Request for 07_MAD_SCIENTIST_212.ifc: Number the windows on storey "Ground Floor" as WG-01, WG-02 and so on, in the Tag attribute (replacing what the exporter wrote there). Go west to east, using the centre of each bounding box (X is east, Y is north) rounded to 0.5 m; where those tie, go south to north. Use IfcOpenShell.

First a look at what the model holds.

```python
import ifcopenshell
import ifcopenshell.util.element
import ifcopenshell.util.placement

model = ifcopenshell.open("07_MAD_SCIENTIST_212.ifc")
print(model.schema)
storey = next(s for s in model.by_type("IfcBuildingStorey") if s.Name == "Ground Floor")
windows = [e for e in ifcopenshell.util.element.get_decomposition(storey) if e.is_a("IfcWindow")]
for e in sorted(windows, key=lambda e: e.id()):
    origin = ifcopenshell.util.placement.get_local_placement(e.ObjectPlacement)[:3, 3]
    print(e.id(), e.Tag, e.Name, origin.round(2) + 0.0, sep=" | ")
```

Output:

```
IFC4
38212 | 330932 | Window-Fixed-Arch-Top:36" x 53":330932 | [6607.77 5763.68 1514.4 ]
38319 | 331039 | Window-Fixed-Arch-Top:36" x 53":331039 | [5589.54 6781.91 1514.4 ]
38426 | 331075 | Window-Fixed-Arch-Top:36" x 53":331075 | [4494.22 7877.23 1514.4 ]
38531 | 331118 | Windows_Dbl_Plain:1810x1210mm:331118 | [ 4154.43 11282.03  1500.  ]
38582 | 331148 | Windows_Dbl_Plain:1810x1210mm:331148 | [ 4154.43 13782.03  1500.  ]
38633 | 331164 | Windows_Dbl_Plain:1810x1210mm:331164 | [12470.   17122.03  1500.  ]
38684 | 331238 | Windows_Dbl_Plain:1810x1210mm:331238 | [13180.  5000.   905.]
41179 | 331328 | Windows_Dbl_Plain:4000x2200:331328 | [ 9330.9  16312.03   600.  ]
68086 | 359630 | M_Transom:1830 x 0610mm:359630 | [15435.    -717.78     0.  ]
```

```python
import ifcopenshell
import ifcopenshell.geom
import ifcopenshell.util.element
import ifcopenshell.util.shape

model = ifcopenshell.open("07_MAD_SCIENTIST_212.ifc")
settings = ifcopenshell.geom.settings()
settings.set("use-world-coords", True)


def centre(element):
    shape = ifcopenshell.geom.create_shape(settings, element)
    return ifcopenshell.util.shape.get_bbox_centroid(shape.geometry)


storey = next(s for s in model.by_type("IfcBuildingStorey") if s.Name == "Ground Floor")
windows = [e for e in ifcopenshell.util.element.get_decomposition(storey) if e.is_a("IfcWindow")]

# Insertion points can sit at a corner or the storey origin, so sort by the geometry (in metres).
centres = {e: centre(e) for e in windows}
windows.sort(key=lambda e: (round(centres[e][0] / 0.5), centres[e][1]))

for i, e in enumerate(windows, start=1):
    number = f"WG-{i:02d}"
    e.Tag = number
    print(e.id(), number)

model.write("07_MAD_SCIENTIST_212_v2.ifc")
```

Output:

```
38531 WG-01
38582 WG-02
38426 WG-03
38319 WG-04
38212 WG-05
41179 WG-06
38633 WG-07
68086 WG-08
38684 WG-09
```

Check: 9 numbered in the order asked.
